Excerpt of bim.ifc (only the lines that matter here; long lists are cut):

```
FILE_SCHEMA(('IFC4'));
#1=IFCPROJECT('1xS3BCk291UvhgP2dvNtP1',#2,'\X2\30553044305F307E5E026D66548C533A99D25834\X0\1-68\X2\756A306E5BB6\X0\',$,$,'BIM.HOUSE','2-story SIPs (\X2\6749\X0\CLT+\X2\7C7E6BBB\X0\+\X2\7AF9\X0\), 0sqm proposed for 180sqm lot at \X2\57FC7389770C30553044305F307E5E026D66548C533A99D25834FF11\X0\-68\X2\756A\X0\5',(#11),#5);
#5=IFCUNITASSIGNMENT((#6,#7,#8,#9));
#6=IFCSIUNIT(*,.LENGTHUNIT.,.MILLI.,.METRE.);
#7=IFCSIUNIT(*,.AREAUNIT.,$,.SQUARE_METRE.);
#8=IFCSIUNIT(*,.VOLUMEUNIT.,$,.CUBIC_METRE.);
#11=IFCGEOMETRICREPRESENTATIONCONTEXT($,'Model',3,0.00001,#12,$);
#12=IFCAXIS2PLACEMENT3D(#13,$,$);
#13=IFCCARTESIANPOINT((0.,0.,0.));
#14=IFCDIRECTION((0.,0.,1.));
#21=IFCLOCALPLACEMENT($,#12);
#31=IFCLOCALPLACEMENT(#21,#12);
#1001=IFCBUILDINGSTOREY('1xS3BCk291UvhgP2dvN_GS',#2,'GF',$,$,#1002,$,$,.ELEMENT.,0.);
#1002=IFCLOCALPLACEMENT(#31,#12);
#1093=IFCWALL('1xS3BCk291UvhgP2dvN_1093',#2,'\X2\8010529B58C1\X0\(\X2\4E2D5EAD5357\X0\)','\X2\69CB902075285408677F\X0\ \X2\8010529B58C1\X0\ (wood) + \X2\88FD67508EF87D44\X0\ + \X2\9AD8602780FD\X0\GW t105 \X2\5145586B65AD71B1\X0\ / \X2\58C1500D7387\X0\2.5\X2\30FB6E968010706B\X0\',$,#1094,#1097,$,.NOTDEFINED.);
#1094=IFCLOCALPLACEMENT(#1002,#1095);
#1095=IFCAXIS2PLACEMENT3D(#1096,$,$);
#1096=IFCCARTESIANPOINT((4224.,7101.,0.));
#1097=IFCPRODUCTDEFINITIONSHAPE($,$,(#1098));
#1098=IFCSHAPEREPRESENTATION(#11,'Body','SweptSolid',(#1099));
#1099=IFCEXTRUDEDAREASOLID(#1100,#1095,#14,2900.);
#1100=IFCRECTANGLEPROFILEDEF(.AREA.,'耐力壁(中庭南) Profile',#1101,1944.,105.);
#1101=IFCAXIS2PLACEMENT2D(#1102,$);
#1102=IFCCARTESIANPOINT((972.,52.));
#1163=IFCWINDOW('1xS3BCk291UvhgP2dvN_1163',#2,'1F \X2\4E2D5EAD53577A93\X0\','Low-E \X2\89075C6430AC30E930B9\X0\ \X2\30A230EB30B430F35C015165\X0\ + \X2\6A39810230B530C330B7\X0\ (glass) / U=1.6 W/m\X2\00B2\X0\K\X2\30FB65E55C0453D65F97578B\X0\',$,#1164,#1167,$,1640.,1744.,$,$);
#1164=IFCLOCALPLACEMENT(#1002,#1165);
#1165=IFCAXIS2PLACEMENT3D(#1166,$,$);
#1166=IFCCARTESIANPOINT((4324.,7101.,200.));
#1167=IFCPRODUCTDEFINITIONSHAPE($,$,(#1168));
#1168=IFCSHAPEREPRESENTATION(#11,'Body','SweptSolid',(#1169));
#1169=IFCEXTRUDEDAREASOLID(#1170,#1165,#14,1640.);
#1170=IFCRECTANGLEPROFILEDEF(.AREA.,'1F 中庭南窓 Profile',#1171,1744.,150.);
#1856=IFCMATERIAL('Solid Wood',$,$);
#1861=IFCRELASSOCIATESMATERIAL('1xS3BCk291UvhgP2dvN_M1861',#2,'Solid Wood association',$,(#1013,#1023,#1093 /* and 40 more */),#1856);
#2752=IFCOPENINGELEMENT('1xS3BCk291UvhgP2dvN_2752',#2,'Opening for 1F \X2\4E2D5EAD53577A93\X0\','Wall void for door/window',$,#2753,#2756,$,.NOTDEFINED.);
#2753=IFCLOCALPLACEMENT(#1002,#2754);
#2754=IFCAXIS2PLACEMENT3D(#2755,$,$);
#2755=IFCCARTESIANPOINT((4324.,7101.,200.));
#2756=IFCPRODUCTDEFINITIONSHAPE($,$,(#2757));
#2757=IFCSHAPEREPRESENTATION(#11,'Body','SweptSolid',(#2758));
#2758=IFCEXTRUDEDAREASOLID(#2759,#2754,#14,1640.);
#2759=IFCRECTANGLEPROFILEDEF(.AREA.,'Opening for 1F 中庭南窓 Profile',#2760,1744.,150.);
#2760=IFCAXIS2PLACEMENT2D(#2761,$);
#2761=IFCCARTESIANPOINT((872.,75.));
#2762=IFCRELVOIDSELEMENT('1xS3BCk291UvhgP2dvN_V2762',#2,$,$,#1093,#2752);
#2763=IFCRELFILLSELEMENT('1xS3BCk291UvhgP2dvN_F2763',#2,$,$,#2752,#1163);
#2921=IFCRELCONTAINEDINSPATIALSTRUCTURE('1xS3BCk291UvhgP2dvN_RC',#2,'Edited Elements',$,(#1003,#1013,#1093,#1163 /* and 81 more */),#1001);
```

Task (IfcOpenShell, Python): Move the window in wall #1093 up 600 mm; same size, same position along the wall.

```python
import numpy as np
import ifcopenshell
import ifcopenshell.api.geometry
import ifcopenshell.util.placement
import ifcopenshell.util.unit

model = ifcopenshell.open("bim.ifc")
unit_scale = ifcopenshell.util.unit.calculate_unit_scale(model)

window = model.by_id(1163)
opening = window.FillsVoids[0].RelatingOpeningElement
dz = 0.6 / unit_scale

shift = np.array([0.0, 0.0, dz])
# The window is not placed relative to its opening, so move both.
for product in (opening, window):
    matrix = ifcopenshell.util.placement.get_local_placement(product.ObjectPlacement)
    matrix[:3, 3] += shift
    ifcopenshell.api.geometry.edit_object_placement(model, product=product, matrix=matrix, is_si=False)

print(f"moved by {dz * unit_scale:+.3f} m")

model.write("bim_updated.ifc")
```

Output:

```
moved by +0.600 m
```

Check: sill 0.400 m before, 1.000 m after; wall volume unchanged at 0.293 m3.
